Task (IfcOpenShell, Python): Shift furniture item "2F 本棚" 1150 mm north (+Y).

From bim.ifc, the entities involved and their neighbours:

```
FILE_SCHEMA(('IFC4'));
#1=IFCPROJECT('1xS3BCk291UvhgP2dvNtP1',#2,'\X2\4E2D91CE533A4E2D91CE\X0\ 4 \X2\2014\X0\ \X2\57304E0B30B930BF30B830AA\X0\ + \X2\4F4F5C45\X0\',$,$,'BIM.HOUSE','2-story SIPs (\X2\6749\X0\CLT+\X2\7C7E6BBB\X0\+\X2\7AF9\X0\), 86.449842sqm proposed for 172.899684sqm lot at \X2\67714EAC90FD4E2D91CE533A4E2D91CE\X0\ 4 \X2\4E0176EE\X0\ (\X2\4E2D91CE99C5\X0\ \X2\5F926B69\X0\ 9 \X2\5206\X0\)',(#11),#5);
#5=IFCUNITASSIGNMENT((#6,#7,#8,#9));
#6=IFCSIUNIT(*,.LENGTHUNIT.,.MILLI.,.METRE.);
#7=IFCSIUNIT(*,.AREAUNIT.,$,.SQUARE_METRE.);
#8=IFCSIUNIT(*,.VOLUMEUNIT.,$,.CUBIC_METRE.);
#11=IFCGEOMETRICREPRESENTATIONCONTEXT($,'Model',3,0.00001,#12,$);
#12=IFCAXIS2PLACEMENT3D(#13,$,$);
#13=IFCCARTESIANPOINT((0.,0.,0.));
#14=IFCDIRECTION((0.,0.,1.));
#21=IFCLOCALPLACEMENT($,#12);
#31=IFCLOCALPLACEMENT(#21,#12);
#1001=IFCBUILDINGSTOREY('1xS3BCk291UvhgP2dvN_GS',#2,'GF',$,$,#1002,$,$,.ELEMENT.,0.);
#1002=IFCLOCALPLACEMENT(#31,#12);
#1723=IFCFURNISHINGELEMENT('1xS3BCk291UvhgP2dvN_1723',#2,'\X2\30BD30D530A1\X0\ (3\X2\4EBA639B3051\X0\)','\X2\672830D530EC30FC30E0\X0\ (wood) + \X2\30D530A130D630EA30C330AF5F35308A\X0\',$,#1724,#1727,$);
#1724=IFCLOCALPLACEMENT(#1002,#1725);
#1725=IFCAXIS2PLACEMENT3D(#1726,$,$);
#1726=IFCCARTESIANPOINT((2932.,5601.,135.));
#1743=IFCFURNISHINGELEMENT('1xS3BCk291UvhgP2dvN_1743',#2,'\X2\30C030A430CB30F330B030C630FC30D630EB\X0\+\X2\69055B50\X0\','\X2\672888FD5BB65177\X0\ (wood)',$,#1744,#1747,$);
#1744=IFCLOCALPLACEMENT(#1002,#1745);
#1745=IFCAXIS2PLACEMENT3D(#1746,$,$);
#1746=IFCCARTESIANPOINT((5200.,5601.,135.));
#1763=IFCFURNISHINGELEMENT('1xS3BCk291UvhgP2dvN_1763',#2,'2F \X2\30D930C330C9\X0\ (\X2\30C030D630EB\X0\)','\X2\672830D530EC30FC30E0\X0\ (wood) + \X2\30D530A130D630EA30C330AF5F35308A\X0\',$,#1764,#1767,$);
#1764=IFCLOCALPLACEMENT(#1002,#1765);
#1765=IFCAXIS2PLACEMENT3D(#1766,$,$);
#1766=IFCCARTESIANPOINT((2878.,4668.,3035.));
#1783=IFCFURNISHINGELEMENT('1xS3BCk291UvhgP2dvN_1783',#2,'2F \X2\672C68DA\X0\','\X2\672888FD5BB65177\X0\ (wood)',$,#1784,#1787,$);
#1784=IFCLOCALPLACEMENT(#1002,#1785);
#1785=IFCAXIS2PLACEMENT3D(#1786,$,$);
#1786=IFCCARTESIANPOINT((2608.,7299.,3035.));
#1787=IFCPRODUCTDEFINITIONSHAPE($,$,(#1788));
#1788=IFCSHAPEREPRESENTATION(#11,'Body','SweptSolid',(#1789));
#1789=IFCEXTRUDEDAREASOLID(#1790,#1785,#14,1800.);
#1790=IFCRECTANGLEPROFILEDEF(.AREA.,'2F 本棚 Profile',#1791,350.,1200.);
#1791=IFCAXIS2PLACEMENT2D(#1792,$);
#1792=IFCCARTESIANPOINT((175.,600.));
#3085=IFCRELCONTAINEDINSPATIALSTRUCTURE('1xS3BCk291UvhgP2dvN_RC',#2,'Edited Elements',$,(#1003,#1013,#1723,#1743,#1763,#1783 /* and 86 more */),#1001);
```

```python
import ifcopenshell
import ifcopenshell.api.geometry
import ifcopenshell.util.placement
import ifcopenshell.util.unit

model = ifcopenshell.open("bim.ifc")
unit_scale = ifcopenshell.util.unit.calculate_unit_scale(model)

item = model.by_guid("1xS3BCk291UvhgP2dvN_1783")
matrix = ifcopenshell.util.placement.get_local_placement(item.ObjectPlacement)
matrix[1, 3] += 1.15 / unit_scale
ifcopenshell.api.geometry.edit_object_placement(model, product=item, matrix=matrix, is_si=False)

print(ifcopenshell.util.placement.get_local_placement(item.ObjectPlacement).round(3) + 0.0)

model.write("bim_updated.ifc")
```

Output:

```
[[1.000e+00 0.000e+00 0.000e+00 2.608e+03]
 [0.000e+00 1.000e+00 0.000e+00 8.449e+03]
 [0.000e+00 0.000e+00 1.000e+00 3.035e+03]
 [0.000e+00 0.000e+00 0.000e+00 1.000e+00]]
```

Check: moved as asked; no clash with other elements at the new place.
